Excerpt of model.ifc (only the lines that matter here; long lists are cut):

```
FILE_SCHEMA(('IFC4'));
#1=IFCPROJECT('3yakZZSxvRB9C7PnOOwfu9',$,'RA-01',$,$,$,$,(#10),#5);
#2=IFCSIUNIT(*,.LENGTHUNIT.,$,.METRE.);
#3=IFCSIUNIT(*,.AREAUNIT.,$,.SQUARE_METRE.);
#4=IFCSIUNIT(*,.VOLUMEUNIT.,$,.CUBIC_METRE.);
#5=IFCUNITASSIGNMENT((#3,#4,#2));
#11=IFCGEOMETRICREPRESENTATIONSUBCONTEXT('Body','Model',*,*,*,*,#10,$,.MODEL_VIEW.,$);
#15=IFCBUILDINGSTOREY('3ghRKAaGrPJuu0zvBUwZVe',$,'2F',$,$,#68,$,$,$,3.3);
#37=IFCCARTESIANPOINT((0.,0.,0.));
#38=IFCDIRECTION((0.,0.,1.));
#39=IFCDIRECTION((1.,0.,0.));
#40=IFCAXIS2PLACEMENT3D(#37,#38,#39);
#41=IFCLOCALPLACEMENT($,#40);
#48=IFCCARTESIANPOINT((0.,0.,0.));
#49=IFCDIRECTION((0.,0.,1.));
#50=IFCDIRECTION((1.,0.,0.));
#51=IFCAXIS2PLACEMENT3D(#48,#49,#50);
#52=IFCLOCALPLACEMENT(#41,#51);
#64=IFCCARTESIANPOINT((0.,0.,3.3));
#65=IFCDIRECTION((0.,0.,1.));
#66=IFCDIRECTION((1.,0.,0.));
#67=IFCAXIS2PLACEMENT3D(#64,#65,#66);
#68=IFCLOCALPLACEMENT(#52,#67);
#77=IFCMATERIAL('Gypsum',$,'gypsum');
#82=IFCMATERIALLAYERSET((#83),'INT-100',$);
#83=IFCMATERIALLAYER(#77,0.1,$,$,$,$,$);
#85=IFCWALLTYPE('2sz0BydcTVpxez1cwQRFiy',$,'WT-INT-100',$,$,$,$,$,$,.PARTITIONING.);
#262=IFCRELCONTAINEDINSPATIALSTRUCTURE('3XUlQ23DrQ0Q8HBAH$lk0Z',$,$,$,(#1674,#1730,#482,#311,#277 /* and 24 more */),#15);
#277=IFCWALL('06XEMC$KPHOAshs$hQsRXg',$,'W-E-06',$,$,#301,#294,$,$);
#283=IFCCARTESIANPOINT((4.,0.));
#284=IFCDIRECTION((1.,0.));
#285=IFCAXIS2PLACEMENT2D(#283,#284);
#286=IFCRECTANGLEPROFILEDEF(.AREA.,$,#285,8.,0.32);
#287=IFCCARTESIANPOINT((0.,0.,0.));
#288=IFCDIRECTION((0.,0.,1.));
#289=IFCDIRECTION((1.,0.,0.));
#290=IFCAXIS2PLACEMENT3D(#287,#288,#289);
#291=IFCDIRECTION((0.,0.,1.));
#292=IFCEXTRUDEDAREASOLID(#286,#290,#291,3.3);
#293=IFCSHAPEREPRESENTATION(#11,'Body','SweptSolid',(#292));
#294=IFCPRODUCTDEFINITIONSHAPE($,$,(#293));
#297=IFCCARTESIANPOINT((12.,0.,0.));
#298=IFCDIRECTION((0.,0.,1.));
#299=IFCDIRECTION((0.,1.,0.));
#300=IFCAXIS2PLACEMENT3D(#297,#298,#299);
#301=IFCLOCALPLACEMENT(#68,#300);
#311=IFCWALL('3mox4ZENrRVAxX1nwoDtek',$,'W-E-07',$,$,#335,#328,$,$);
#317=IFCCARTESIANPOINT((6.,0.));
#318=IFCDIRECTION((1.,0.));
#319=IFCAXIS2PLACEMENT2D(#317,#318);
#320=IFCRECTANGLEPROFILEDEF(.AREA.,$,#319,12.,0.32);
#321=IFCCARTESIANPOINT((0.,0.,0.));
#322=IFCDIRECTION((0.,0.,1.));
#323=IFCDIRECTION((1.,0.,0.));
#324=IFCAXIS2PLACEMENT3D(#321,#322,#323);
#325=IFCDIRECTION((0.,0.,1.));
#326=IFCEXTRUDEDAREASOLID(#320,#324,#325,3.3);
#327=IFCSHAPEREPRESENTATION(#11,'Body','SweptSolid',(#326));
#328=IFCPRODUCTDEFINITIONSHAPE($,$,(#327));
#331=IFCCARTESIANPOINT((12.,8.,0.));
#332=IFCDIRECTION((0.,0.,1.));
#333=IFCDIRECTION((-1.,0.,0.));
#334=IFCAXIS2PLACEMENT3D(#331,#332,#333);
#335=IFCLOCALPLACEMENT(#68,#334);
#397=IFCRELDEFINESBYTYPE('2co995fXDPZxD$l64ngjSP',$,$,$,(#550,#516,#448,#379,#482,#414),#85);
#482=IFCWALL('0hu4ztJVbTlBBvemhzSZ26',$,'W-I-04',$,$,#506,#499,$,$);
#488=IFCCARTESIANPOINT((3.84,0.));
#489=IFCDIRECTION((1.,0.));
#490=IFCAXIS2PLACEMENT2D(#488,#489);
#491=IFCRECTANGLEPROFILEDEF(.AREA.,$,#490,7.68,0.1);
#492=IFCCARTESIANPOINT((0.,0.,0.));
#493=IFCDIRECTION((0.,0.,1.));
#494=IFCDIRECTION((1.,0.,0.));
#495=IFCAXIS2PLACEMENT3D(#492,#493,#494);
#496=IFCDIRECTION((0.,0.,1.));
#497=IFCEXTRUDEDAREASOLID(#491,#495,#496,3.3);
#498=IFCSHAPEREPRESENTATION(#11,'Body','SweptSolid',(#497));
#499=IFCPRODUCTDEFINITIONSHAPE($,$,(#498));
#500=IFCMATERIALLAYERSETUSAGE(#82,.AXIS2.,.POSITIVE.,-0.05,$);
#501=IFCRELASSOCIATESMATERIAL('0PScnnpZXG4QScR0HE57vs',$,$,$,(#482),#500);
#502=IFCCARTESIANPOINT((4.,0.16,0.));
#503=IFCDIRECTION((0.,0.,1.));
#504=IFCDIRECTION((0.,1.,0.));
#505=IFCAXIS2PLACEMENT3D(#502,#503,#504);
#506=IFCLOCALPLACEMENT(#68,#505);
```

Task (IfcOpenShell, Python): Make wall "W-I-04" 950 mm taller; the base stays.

```python
import ifcopenshell
import ifcopenshell.geom
import ifcopenshell.util.representation
import ifcopenshell.util.shape

model = ifcopenshell.open("model.ifc")
settings = ifcopenshell.geom.settings()


def volume(element):
    """Net volume in cubic metres, openings subtracted."""
    shape = ifcopenshell.geom.create_shape(settings, element)
    return ifcopenshell.util.shape.get_volume(shape.geometry)


wall = model.by_guid("0hu4ztJVbTlBBvemhzSZ26")
before = volume(wall)

body = ifcopenshell.util.representation.get_representation(wall, "Model", "Body")
solid = body.Items[0]
old_height = solid.Depth
solid.Depth += 0.95
after = volume(wall)

print(f"height {old_height:g} -> {solid.Depth:g}, volume {before:.3f} -> {after:.3f} m3")

model.write("model_updated.ifc")
```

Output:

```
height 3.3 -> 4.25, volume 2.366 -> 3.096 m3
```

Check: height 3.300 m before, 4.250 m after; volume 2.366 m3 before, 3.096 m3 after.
